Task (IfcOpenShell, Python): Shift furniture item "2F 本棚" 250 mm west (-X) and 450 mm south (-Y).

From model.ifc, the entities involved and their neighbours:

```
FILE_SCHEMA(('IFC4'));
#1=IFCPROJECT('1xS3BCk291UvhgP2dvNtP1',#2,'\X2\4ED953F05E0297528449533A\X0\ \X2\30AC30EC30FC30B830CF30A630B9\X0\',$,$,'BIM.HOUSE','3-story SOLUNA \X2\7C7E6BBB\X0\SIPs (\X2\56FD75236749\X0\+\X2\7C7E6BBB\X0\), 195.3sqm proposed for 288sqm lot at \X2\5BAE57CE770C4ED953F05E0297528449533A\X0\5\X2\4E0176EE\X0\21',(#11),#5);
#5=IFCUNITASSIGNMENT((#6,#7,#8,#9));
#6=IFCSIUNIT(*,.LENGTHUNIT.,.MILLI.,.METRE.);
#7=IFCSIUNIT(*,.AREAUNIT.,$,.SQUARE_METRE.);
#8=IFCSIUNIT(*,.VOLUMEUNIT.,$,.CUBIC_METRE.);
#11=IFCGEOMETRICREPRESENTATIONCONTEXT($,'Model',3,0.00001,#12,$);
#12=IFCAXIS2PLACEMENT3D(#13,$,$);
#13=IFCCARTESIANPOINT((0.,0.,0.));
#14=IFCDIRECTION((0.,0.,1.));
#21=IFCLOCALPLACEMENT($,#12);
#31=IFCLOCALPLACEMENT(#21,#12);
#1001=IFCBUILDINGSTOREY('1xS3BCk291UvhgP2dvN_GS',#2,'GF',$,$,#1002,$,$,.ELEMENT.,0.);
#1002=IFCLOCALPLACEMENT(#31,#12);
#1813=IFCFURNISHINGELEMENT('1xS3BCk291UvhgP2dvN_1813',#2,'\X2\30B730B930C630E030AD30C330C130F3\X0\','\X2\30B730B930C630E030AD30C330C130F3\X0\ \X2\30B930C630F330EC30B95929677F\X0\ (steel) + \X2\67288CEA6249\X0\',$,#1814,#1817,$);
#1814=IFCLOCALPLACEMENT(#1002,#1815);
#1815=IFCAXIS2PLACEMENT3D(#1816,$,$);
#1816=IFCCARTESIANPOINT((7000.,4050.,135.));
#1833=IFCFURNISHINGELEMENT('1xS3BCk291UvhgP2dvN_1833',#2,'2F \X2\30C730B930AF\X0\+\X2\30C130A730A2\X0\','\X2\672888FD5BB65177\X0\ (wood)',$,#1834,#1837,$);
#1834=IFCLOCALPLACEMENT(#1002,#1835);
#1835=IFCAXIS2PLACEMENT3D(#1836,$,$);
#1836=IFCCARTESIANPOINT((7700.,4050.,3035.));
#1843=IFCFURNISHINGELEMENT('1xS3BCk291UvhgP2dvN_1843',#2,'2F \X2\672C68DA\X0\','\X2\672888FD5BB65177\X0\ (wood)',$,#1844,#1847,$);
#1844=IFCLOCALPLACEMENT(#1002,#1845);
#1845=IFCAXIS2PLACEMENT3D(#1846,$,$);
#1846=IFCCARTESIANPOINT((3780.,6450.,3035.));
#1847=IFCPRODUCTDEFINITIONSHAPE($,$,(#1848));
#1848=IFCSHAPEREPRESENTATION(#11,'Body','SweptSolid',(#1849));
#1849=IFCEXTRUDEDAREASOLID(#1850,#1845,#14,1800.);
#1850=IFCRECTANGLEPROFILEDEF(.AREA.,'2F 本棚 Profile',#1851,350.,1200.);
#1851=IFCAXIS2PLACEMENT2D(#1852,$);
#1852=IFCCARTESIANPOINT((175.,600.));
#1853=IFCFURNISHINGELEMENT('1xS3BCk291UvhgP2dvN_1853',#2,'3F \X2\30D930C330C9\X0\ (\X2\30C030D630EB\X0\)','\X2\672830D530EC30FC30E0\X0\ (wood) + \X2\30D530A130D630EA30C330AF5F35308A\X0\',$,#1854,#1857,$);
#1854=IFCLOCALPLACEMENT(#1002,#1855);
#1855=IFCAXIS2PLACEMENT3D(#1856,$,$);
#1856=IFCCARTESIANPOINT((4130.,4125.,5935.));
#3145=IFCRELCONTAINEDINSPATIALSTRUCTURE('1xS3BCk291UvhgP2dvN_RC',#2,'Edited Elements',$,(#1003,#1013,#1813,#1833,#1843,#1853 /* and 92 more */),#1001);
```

```python
import ifcopenshell
import ifcopenshell.api.geometry
import ifcopenshell.util.placement

model = ifcopenshell.open("model.ifc")

item = model.by_id(1843)
matrix = ifcopenshell.util.placement.get_local_placement(item.ObjectPlacement)
matrix[0, 3] -= 250.0
matrix[1, 3] -= 450.0
ifcopenshell.api.geometry.edit_object_placement(model, product=item, matrix=matrix, is_si=False)

print(ifcopenshell.util.placement.get_local_placement(item.ObjectPlacement).round(3) + 0.0)

model.write("model-out.ifc")
```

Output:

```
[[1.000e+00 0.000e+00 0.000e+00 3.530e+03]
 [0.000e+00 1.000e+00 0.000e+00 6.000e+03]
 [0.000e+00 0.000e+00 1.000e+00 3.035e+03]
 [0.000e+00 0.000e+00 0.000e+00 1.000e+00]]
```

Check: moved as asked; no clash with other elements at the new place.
